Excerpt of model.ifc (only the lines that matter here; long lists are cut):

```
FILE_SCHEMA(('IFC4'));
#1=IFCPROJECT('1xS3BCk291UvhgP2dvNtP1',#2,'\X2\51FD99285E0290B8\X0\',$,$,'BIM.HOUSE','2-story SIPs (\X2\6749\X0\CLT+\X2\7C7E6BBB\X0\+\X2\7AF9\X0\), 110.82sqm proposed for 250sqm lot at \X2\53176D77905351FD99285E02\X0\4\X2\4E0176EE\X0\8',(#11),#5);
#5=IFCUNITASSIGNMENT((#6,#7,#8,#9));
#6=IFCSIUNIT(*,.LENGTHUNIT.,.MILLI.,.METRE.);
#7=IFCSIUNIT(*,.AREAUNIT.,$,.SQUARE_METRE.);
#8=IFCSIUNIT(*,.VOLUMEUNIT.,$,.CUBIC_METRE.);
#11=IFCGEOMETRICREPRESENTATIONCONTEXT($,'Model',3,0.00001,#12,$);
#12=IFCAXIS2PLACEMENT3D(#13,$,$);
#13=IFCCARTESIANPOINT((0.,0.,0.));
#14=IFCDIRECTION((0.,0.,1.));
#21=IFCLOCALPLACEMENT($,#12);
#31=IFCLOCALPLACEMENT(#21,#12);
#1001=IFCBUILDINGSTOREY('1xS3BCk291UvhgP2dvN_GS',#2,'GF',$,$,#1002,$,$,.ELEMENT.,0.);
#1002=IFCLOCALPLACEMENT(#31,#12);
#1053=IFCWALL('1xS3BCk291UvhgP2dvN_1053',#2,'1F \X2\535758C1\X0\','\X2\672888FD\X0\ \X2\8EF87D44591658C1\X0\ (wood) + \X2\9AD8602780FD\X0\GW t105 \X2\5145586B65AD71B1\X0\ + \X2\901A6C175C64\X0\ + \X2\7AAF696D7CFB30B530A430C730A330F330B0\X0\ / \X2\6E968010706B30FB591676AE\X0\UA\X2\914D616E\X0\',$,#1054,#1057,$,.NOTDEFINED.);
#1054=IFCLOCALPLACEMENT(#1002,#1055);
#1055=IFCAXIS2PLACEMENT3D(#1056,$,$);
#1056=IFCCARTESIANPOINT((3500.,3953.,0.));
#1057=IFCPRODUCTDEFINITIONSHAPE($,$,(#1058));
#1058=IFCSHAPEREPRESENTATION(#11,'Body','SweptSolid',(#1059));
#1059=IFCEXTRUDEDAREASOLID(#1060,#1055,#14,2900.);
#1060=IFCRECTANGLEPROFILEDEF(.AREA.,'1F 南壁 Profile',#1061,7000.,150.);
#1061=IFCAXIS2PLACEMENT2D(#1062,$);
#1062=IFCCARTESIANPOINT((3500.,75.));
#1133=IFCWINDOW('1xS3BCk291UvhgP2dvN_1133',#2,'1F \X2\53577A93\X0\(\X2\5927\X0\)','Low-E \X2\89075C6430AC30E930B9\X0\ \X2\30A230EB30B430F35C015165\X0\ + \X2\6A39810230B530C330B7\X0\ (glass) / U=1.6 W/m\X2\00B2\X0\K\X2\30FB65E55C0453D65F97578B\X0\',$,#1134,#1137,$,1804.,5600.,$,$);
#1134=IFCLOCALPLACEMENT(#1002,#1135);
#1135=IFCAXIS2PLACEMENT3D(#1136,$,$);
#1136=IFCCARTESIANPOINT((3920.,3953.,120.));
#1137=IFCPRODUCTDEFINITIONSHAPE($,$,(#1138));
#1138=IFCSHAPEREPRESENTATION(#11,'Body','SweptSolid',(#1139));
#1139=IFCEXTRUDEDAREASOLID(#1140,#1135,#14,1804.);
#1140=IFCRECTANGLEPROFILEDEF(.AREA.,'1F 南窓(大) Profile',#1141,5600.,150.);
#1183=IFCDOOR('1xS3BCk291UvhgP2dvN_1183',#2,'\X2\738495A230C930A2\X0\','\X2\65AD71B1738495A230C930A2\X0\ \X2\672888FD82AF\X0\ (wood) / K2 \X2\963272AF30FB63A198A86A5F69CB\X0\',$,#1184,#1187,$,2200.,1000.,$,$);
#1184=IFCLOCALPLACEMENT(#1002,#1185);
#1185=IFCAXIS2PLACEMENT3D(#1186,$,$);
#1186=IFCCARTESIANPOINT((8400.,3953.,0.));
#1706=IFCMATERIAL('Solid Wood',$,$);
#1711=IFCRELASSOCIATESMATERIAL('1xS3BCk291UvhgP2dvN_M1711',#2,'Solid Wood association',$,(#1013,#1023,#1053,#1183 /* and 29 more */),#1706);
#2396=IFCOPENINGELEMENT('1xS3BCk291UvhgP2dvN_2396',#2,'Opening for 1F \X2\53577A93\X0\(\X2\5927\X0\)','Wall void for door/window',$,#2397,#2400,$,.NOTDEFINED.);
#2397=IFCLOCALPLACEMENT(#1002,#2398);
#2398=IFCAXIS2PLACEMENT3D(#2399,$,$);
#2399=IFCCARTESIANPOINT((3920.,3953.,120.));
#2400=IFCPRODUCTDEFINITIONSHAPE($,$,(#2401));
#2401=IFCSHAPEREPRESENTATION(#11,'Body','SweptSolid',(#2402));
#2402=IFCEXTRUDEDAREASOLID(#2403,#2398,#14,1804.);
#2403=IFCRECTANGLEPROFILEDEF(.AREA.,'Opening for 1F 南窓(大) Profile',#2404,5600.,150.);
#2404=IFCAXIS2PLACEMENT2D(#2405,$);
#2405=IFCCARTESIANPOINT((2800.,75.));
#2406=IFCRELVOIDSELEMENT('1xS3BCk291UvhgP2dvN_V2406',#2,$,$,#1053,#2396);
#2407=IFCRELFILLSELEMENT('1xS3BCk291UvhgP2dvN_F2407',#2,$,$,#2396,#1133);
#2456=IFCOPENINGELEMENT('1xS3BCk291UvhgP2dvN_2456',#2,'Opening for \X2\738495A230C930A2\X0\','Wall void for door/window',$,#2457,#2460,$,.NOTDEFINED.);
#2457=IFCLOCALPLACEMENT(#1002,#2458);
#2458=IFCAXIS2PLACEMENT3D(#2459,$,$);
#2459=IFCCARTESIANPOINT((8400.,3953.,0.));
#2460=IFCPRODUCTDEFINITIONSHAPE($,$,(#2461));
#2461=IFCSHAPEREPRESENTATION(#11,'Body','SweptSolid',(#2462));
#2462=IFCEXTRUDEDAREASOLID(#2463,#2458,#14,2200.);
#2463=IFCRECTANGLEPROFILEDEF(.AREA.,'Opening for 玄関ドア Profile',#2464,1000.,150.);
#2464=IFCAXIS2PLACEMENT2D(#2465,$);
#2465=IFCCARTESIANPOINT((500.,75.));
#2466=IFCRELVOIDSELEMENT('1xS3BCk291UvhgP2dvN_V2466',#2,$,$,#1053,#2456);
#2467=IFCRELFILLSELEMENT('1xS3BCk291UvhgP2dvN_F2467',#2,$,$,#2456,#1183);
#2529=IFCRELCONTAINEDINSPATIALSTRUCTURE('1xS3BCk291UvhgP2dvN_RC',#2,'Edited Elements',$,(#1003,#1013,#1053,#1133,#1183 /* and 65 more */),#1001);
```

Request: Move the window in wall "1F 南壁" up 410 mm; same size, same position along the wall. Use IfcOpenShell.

```python
import numpy as np
import ifcopenshell
import ifcopenshell.api.geometry
import ifcopenshell.util.placement
import ifcopenshell.util.unit

model = ifcopenshell.open("model.ifc")
unit_scale = ifcopenshell.util.unit.calculate_unit_scale(model)

window = model.by_guid("1xS3BCk291UvhgP2dvN_1133")
opening = window.FillsVoids[0].RelatingOpeningElement
dz = 410.0

shift = np.array([0.0, 0.0, dz])
# The window is not placed relative to its opening, so move both.
for product in (opening, window):
    matrix = ifcopenshell.util.placement.get_local_placement(product.ObjectPlacement)
    matrix[:3, 3] += shift
    ifcopenshell.api.geometry.edit_object_placement(model, product=product, matrix=matrix, is_si=False)

print(f"moved by {dz * unit_scale:+.3f} m")

model.write("model_updated.ifc")
```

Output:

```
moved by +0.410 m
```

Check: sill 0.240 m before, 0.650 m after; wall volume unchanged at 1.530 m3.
